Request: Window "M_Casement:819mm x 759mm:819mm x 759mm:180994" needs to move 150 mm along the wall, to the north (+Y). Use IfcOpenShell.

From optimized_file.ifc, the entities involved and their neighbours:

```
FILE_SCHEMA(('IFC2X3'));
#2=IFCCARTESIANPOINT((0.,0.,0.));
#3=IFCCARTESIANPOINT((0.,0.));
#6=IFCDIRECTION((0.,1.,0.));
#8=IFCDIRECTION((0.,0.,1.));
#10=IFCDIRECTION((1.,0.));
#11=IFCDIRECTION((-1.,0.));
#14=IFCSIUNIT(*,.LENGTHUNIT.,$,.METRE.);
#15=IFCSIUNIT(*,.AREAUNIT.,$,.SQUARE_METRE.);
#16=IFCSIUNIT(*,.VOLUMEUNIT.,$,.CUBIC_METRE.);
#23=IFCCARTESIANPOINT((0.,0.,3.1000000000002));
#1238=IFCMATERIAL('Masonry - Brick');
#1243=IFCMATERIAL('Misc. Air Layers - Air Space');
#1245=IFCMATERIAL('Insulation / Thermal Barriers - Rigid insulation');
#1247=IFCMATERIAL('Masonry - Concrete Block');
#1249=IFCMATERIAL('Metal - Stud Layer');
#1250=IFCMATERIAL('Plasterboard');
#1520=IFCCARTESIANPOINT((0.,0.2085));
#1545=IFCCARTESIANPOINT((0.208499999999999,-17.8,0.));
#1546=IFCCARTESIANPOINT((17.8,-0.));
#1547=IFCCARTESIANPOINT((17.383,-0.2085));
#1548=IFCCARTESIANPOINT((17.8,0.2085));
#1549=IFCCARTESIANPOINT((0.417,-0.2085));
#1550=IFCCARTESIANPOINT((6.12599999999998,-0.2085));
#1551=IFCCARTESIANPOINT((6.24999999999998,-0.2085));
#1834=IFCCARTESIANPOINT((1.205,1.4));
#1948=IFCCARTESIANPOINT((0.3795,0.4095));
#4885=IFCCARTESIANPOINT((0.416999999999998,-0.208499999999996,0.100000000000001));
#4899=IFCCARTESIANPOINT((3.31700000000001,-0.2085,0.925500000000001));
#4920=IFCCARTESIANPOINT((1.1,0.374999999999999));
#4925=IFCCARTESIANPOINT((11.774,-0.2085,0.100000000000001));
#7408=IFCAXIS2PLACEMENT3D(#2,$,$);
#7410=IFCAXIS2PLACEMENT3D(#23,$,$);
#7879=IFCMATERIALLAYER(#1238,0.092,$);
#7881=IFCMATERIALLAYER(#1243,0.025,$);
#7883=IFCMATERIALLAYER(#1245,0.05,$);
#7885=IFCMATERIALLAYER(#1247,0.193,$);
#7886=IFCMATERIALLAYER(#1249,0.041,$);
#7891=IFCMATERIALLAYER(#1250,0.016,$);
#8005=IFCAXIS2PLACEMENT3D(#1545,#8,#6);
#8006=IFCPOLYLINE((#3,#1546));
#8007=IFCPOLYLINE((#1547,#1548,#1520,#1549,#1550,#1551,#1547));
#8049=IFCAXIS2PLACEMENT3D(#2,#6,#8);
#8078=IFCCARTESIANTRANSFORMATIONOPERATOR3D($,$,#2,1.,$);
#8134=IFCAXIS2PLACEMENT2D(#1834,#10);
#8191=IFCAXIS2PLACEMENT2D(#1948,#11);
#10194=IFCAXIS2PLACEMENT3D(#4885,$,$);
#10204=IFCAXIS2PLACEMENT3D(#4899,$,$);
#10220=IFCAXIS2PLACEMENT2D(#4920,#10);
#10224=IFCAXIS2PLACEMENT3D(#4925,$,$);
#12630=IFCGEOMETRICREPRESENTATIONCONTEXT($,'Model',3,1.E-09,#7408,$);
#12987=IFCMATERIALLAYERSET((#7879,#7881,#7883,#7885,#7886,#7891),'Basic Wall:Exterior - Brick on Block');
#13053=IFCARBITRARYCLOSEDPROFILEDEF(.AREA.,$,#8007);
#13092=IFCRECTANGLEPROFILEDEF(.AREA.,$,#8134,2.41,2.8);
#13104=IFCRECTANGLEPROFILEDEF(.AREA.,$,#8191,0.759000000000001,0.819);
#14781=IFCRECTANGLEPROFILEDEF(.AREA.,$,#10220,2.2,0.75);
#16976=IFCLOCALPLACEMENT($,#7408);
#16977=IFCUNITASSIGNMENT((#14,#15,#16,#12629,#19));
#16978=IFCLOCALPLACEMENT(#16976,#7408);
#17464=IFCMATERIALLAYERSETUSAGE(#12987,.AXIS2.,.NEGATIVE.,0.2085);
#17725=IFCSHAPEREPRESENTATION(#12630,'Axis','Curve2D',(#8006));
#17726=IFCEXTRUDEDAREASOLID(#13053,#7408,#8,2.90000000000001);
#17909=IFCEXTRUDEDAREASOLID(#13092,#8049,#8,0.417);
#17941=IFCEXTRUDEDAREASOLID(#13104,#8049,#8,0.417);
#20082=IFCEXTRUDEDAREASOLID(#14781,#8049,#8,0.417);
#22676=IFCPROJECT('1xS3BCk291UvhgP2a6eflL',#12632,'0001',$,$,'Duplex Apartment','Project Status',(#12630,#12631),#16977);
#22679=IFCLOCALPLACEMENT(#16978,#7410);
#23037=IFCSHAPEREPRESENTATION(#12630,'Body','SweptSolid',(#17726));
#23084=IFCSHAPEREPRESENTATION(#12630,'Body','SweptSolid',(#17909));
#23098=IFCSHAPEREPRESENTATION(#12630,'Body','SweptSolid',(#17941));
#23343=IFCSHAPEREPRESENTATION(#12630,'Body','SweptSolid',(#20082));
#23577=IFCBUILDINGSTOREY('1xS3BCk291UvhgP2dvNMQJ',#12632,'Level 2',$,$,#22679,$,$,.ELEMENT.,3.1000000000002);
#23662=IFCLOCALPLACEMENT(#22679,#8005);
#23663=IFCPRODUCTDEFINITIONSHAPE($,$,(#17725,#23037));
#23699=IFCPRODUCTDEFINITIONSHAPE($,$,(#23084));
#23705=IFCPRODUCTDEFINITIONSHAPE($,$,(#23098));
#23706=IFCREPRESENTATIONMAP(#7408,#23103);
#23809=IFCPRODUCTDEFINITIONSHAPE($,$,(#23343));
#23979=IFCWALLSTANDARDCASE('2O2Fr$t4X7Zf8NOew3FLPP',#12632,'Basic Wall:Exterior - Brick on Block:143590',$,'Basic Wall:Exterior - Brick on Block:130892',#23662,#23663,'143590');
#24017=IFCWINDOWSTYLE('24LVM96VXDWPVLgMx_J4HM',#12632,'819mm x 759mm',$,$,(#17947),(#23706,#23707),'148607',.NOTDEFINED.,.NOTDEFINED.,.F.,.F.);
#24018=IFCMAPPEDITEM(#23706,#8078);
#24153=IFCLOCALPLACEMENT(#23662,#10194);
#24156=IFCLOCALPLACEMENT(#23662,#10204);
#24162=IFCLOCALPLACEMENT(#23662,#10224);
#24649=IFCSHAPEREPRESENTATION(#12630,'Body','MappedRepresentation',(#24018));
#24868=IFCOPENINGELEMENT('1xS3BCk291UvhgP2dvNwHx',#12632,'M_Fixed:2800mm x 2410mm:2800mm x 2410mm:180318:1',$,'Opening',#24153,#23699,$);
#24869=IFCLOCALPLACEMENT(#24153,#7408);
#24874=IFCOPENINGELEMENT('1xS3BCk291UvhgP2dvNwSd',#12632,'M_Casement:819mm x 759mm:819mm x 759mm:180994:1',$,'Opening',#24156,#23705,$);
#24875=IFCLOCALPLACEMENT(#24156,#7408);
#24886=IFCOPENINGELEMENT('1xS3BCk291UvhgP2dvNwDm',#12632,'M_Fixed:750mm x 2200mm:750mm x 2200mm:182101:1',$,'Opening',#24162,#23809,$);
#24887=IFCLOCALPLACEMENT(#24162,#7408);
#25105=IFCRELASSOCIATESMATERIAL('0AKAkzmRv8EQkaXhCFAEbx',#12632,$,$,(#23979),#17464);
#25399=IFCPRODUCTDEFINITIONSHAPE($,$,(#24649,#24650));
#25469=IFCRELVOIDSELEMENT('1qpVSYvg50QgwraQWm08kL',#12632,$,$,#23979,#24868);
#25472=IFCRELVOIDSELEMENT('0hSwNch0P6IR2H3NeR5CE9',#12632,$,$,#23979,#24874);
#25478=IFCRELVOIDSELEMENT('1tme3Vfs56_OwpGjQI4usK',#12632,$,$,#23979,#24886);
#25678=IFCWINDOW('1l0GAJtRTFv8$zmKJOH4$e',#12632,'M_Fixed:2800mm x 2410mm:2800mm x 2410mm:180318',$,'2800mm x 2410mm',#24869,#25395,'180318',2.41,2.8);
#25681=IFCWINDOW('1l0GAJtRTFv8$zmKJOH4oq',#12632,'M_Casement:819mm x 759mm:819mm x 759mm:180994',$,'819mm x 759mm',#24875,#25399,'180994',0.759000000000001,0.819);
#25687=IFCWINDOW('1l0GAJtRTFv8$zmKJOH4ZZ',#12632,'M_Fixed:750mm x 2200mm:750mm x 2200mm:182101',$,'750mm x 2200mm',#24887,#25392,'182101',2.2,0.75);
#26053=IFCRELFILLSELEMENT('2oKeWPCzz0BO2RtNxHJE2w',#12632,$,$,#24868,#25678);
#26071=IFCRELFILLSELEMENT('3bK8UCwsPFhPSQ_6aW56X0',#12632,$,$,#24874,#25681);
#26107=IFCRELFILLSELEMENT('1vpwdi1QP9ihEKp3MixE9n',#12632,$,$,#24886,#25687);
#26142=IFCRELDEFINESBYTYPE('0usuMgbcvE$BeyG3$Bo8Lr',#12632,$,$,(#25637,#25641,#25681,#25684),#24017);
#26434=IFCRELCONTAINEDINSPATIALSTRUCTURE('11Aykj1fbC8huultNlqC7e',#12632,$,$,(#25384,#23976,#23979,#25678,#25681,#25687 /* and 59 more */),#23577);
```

```python
import ifcopenshell
import ifcopenshell.api.geometry
import ifcopenshell.util.placement
import ifcopenshell.util.unit

model = ifcopenshell.open("optimized_file.ifc")
unit_scale = ifcopenshell.util.unit.calculate_unit_scale(model)

window = model.by_guid("1l0GAJtRTFv8$zmKJOH4oq")
opening = window.FillsVoids[0].RelatingOpeningElement
wall = opening.VoidsElements[0].RelatingBuildingElement

wall_matrix = ifcopenshell.util.placement.get_local_placement(wall.ObjectPlacement)
shift = wall_matrix[:3, 0] * 0.15 / unit_scale
before = ifcopenshell.util.placement.get_local_placement(window.ObjectPlacement)[:3, 3].copy()

# The window is placed relative to its opening, so it follows when the opening moves.
matrix = ifcopenshell.util.placement.get_local_placement(opening.ObjectPlacement)
matrix[:3, 3] += shift
ifcopenshell.api.geometry.edit_object_placement(
    model, product=opening, matrix=matrix, is_si=False, should_transform_children=True
)

after = ifcopenshell.util.placement.get_local_placement(window.ObjectPlacement)[:3, 3]
print("window moved by", (after - before).round(3) + 0.0)

model.write("optimized_file_updated.ifc")
```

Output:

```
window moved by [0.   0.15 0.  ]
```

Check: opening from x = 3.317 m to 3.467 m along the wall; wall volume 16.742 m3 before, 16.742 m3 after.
